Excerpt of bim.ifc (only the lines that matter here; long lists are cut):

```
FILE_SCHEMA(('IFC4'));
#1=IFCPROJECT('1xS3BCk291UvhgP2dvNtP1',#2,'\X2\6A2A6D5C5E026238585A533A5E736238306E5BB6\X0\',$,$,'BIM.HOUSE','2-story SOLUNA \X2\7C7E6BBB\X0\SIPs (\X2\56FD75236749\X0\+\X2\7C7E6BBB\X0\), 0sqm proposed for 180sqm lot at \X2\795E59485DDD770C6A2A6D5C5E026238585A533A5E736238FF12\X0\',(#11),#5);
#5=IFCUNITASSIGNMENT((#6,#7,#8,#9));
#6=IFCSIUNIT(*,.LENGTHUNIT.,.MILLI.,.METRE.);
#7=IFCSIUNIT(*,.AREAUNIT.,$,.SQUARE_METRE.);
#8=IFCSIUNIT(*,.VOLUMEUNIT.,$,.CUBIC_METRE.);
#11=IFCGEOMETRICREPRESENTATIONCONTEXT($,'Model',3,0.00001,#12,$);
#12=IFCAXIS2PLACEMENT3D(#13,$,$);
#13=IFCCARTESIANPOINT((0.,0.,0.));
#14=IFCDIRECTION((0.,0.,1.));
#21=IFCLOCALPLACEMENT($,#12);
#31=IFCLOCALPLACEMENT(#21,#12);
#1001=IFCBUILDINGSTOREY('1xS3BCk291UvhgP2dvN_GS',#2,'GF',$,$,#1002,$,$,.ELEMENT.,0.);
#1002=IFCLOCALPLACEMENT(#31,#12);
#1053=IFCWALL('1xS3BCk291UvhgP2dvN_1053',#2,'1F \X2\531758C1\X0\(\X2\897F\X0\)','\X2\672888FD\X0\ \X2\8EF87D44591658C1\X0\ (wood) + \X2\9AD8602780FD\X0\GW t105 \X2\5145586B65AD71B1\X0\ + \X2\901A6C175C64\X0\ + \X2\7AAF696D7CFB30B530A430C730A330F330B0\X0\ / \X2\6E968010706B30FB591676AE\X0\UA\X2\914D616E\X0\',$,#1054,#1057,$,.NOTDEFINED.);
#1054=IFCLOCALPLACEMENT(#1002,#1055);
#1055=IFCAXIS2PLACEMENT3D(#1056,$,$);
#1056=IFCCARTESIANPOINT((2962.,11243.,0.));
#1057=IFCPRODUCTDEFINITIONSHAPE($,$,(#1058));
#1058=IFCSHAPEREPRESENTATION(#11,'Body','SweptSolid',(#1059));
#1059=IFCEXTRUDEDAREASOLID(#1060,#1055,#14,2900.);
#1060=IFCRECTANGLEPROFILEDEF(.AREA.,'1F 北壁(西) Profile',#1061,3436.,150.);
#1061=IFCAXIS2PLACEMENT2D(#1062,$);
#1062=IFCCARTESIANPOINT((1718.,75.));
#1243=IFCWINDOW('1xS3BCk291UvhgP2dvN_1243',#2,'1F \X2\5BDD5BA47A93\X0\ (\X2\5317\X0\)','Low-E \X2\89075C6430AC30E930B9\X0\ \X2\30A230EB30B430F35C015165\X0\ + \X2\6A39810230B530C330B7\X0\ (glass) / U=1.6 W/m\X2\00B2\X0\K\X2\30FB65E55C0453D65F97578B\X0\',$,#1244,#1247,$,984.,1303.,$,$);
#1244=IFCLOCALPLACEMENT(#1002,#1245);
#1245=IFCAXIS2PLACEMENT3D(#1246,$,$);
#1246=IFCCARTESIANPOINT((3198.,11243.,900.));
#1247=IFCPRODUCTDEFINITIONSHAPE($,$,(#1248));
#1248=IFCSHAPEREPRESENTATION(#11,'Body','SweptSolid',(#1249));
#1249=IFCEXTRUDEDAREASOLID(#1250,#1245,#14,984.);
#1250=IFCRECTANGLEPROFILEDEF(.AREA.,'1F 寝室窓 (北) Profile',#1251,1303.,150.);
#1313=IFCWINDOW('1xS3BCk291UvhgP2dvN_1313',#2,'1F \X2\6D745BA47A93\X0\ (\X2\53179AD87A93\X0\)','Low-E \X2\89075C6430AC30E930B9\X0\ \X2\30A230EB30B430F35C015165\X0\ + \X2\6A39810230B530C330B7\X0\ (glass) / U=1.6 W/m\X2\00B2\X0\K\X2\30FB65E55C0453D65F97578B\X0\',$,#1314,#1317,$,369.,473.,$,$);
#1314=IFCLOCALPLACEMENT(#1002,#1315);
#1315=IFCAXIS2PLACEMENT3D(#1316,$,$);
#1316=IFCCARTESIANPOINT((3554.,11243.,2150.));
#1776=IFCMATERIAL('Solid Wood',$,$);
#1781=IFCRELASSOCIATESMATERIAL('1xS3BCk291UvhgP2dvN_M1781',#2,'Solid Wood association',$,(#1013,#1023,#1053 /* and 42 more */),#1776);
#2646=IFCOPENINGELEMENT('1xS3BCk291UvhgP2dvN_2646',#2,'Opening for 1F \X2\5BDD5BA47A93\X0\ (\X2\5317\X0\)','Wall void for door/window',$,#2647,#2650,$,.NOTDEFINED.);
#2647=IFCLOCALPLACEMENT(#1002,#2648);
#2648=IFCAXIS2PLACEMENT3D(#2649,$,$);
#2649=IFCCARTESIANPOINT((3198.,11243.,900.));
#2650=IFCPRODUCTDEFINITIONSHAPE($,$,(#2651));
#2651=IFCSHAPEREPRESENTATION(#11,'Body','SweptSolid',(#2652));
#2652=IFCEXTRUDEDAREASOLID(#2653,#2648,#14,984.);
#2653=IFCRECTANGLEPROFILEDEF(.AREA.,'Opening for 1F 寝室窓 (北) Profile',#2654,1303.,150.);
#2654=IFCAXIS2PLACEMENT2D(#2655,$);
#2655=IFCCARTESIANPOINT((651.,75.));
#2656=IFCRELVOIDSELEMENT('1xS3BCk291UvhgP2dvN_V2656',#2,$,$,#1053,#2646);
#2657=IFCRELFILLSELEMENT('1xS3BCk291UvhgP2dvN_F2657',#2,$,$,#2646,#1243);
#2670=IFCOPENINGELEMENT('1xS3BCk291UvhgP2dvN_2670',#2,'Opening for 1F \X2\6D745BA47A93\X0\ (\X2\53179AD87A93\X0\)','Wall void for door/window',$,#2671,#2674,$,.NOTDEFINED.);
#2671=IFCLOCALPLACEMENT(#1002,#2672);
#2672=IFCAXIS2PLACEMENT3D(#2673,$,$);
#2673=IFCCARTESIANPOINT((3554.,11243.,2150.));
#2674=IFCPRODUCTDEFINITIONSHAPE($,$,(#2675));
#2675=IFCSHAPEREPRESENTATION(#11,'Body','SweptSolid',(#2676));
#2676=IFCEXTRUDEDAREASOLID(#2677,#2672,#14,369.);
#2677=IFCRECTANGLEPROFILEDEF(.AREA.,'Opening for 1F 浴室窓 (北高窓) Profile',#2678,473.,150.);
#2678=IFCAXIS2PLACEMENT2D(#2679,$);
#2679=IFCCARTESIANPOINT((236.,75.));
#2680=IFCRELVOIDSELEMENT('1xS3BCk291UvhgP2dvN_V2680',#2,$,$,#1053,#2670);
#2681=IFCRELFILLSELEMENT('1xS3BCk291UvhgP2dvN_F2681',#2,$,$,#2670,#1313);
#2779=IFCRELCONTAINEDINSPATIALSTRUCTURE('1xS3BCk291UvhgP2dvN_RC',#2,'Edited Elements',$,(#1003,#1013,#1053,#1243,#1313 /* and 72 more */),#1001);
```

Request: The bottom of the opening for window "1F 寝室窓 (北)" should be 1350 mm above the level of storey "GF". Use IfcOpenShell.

```python
import numpy as np
import ifcopenshell
import ifcopenshell.api.geometry
import ifcopenshell.geom
import ifcopenshell.util.element
import ifcopenshell.util.placement
import ifcopenshell.util.shape
import ifcopenshell.util.unit

model = ifcopenshell.open("bim.ifc")
unit_scale = ifcopenshell.util.unit.calculate_unit_scale(model)

window = model.by_guid("1xS3BCk291UvhgP2dvN_1243")
opening = window.FillsVoids[0].RelatingOpeningElement
storey = ifcopenshell.util.element.get_container(window, ifc_class="IfcBuildingStorey")
level = ifcopenshell.util.placement.get_local_placement(storey.ObjectPlacement)[2, 3]

# The opening's origin need not be at the sill, so measure its lowest point.
shape = ifcopenshell.geom.create_shape(ifcopenshell.geom.settings(), opening)
bottom = ifcopenshell.util.shape.get_shape_bottom_elevation(shape, shape.geometry) / unit_scale
dz = level + 1350.0 - bottom

shift = np.array([0.0, 0.0, dz])
# The window is not placed relative to its opening, so move both.
for product in (opening, window):
    matrix = ifcopenshell.util.placement.get_local_placement(product.ObjectPlacement)
    matrix[:3, 3] += shift
    ifcopenshell.api.geometry.edit_object_placement(model, product=product, matrix=matrix, is_si=False)

print(f"moved by {dz * unit_scale:+.3f} m")

model.write("bim_v2.ifc")
```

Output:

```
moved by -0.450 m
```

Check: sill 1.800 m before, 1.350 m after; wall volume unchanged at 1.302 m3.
